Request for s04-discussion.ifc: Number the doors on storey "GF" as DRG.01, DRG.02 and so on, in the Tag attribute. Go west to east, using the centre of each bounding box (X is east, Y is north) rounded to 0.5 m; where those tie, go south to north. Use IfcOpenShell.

First a look at what the model holds.

```python
import ifcopenshell
import ifcopenshell.util.element
import ifcopenshell.util.placement

model = ifcopenshell.open("s04-discussion.ifc")
print(model.schema)
storey = next(s for s in model.by_type("IfcBuildingStorey") if s.Name == "GF")
doors = [e for e in ifcopenshell.util.element.get_decomposition(storey) if e.is_a("IfcDoor")]
for e in sorted(doors, key=lambda e: e.id()):
    origin = ifcopenshell.util.placement.get_local_placement(e.ObjectPlacement)[:3, 3]
    print(e.id(), e.Tag, e.Name, origin.round(2) + 0.0, sep=" | ")
```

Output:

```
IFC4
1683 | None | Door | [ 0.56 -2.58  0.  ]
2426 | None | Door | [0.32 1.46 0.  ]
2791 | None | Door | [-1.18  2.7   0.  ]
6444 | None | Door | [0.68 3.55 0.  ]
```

```python
import ifcopenshell
import ifcopenshell.geom
import ifcopenshell.util.element
import ifcopenshell.util.shape

model = ifcopenshell.open("s04-discussion.ifc")
settings = ifcopenshell.geom.settings()
settings.set("use-world-coords", True)


def centre(element):
    shape = ifcopenshell.geom.create_shape(settings, element)
    return ifcopenshell.util.shape.get_bbox_centroid(shape.geometry)


storey = next(s for s in model.by_type("IfcBuildingStorey") if s.Name == "GF")
doors = [e for e in ifcopenshell.util.element.get_decomposition(storey) if e.is_a("IfcDoor")]

# Insertion points can sit at a corner or the storey origin, so sort by the geometry (in metres).
centres = {e: centre(e) for e in doors}
doors.sort(key=lambda e: (round(centres[e][0] / 0.5), centres[e][1]))

for i, e in enumerate(doors, start=1):
    number = f"DRG.{i:02d}"
    e.Tag = number
    print(e.id(), number)

model.write("s04-discussion_v2.ifc")
```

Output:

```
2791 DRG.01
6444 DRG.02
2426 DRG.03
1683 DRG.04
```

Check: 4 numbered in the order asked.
